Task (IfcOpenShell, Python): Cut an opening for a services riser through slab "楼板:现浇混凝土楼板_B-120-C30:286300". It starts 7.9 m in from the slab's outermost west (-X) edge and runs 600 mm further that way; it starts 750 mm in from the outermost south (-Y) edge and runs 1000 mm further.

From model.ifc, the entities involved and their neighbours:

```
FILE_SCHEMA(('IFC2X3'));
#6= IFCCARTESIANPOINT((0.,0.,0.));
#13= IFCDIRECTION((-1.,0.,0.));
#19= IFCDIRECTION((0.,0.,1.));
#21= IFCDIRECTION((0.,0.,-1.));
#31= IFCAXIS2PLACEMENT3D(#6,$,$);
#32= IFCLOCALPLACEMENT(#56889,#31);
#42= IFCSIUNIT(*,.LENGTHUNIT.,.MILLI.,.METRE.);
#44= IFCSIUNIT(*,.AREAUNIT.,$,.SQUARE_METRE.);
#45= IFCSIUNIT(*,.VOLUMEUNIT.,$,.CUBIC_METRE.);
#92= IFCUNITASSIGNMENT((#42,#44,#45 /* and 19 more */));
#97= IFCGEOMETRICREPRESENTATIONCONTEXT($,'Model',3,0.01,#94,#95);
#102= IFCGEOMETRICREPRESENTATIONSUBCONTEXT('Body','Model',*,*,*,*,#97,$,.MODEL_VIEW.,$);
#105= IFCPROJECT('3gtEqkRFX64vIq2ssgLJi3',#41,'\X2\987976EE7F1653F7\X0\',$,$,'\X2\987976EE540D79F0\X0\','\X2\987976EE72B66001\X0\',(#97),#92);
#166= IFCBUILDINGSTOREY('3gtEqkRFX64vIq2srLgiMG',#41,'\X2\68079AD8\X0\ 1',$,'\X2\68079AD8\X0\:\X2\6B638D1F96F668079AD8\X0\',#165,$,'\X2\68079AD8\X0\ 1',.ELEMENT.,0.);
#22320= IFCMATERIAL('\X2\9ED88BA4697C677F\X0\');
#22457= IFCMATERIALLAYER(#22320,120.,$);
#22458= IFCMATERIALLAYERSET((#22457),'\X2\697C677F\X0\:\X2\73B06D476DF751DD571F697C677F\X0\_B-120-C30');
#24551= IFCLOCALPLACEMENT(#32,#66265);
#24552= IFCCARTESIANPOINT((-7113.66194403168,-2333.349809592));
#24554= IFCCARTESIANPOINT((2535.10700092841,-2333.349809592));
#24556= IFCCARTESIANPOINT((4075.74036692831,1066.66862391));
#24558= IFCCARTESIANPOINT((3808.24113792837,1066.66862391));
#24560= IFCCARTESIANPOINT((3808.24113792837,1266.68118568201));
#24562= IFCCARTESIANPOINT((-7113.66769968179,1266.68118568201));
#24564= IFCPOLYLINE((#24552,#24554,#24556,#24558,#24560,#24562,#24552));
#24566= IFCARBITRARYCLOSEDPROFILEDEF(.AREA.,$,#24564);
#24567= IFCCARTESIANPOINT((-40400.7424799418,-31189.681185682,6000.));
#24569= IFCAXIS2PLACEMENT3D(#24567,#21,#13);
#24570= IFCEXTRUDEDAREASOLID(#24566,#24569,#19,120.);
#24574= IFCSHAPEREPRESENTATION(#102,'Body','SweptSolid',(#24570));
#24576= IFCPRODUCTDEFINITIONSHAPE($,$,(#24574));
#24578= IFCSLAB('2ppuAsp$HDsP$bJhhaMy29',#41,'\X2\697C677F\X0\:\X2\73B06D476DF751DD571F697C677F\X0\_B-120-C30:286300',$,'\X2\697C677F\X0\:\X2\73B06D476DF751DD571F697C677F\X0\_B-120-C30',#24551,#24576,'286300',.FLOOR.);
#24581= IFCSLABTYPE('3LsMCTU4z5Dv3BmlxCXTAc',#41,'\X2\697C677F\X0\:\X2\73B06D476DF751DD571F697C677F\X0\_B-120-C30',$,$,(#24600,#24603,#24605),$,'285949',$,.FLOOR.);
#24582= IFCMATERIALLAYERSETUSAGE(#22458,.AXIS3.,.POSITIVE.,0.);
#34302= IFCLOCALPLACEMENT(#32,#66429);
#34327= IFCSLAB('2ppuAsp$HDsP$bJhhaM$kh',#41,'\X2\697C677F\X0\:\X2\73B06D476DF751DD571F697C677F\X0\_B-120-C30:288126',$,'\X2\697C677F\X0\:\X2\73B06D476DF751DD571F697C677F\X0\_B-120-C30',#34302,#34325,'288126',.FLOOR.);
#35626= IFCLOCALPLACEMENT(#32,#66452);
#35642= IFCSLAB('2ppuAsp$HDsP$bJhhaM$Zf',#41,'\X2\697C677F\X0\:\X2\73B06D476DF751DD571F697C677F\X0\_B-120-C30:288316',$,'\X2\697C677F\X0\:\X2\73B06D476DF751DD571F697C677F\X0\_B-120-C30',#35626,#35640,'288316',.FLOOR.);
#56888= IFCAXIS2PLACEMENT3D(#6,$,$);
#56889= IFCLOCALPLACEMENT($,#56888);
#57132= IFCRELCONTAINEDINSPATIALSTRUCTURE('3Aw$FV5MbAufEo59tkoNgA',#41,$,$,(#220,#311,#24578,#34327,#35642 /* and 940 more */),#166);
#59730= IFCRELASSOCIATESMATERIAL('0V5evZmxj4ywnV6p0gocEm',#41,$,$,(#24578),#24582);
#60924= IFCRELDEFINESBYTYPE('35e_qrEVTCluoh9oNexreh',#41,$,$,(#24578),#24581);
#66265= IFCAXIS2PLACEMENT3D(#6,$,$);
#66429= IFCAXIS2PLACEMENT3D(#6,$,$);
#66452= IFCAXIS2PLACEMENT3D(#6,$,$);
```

```python
import numpy as np
import ifcopenshell
import ifcopenshell.api.feature
import ifcopenshell.api.geometry
import ifcopenshell.api.root
import ifcopenshell.geom
import ifcopenshell.util.placement
import ifcopenshell.util.representation
import ifcopenshell.util.shape
import ifcopenshell.util.unit

model = ifcopenshell.open("model.ifc")
unit_scale = ifcopenshell.util.unit.calculate_unit_scale(model)
settings = ifcopenshell.geom.settings()


def volume(element):
    """Net volume in cubic metres, openings subtracted."""
    shape = ifcopenshell.geom.create_shape(settings, element)
    return ifcopenshell.util.shape.get_volume(shape.geometry)


slab = model.by_guid("2ppuAsp$HDsP$bJhhaMy29")
before = volume(slab)

# Extent in the slab's own axes, in metres. The edges named are its -X and -Y sides.
slab_shape = ifcopenshell.geom.create_shape(settings, slab)
vertices = ifcopenshell.util.shape.get_vertices(slab_shape.geometry)
x_min, y_min, bottom = vertices.min(axis=0)
top = vertices[:, 2].max()

opening = ifcopenshell.api.root.create_entity(model, ifc_class="IfcOpeningElement", name="Services riser opening")
context = ifcopenshell.util.representation.get_context(model, "Model", "Body", "MODEL_VIEW")
width, depth = 0.6, 1
outline = [(0.0, 0.0), (width, 0.0), (width, depth), (0.0, depth), (0.0, 0.0)]
# Overshoot both faces by 50 mm so the cut is clean.
shape = ifcopenshell.api.geometry.add_slab_representation(
    model, context=context, depth=top - bottom + 0.1, polyline=outline
)
ifcopenshell.api.geometry.assign_representation(model, product=opening, representation=shape)

matrix = ifcopenshell.util.placement.get_local_placement(slab.ObjectPlacement)
matrix[:, 3] = matrix @ np.append(np.array([x_min + 7.9, y_min + 0.75, bottom - 0.05]) / unit_scale, 1.0)
ifcopenshell.api.geometry.edit_object_placement(model, product=opening, matrix=matrix, is_si=False)
ifcopenshell.api.feature.add_feature(model, feature=opening, element=slab)

after = volume(slab)

print(f"slab volume {before:.3f} -> {after:.3f} m3")

model.write("model_updated.ifc")
```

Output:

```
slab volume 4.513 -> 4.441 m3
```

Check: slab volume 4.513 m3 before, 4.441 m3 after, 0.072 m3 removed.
